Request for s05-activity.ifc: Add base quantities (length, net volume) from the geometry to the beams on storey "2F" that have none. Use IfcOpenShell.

First a look at what the model holds.

```python
import ifcopenshell
import ifcopenshell.util.element
import ifcopenshell.util.unit

model = ifcopenshell.open("s05-activity.ifc")
print(model.schema)
for unit_type in ("LENGTHUNIT", "AREAUNIT", "VOLUMEUNIT"):
    print(unit_type, ifcopenshell.util.unit.calculate_unit_scale(model, unit_type))
storey = next(s for s in model.by_type("IfcBuildingStorey") if s.Name == "2F")
beams = [e for e in ifcopenshell.util.element.get_decomposition(storey) if e.is_a("IfcBeam")]
for e in sorted(beams, key=lambda e: e.id()):
    print(e.id(), e.is_a(), e.Name, list(ifcopenshell.util.element.get_psets(e, qtos_only=True)), sep=" | ")
```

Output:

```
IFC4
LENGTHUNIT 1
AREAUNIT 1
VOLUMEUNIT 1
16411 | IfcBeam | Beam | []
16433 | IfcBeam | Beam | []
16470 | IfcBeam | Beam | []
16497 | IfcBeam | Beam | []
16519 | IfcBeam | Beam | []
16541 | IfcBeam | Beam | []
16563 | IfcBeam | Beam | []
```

```python
import ifcopenshell
import ifcopenshell.api.pset
import ifcopenshell.geom
import ifcopenshell.util.element
import ifcopenshell.util.shape
import ifcopenshell.util.unit

model = ifcopenshell.open("s05-activity.ifc")
unit_scale = ifcopenshell.util.unit.calculate_unit_scale(model)
volume_scale = ifcopenshell.util.unit.calculate_unit_scale(model, "VOLUMEUNIT")
settings = ifcopenshell.geom.settings()

storey = next(s for s in model.by_type("IfcBuildingStorey") if s.Name == "2F")
beams = [e for e in ifcopenshell.util.element.get_decomposition(storey) if e.is_a("IfcBeam")]

for e in sorted(beams, key=lambda e: e.id()):
    if ifcopenshell.util.element.get_psets(e, qtos_only=True, should_inherit=False):
        continue
    # Geometry comes back in metres, in the element's own axes.
    shape = ifcopenshell.geom.create_shape(settings, e)
    values = {
        "Length": ifcopenshell.util.shape.get_max_xyz(shape.geometry) / unit_scale,
        "NetVolume": ifcopenshell.util.shape.get_volume(shape.geometry) / volume_scale,
    }
    qto = ifcopenshell.api.pset.add_qto(model, product=e, name="Qto_BeamBaseQuantities")
    ifcopenshell.api.pset.edit_qto(model, qto=qto, properties=values)
    print(e.id(), {k: round(v, 3) for k, v in values.items()})

model.write("s05-activity-out.ifc")
```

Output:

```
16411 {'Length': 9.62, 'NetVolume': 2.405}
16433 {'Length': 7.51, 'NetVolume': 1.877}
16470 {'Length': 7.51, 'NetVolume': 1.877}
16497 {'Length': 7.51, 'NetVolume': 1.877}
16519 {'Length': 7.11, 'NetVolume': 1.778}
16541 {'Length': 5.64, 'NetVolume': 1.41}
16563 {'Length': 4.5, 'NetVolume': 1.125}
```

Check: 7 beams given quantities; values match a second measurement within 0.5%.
